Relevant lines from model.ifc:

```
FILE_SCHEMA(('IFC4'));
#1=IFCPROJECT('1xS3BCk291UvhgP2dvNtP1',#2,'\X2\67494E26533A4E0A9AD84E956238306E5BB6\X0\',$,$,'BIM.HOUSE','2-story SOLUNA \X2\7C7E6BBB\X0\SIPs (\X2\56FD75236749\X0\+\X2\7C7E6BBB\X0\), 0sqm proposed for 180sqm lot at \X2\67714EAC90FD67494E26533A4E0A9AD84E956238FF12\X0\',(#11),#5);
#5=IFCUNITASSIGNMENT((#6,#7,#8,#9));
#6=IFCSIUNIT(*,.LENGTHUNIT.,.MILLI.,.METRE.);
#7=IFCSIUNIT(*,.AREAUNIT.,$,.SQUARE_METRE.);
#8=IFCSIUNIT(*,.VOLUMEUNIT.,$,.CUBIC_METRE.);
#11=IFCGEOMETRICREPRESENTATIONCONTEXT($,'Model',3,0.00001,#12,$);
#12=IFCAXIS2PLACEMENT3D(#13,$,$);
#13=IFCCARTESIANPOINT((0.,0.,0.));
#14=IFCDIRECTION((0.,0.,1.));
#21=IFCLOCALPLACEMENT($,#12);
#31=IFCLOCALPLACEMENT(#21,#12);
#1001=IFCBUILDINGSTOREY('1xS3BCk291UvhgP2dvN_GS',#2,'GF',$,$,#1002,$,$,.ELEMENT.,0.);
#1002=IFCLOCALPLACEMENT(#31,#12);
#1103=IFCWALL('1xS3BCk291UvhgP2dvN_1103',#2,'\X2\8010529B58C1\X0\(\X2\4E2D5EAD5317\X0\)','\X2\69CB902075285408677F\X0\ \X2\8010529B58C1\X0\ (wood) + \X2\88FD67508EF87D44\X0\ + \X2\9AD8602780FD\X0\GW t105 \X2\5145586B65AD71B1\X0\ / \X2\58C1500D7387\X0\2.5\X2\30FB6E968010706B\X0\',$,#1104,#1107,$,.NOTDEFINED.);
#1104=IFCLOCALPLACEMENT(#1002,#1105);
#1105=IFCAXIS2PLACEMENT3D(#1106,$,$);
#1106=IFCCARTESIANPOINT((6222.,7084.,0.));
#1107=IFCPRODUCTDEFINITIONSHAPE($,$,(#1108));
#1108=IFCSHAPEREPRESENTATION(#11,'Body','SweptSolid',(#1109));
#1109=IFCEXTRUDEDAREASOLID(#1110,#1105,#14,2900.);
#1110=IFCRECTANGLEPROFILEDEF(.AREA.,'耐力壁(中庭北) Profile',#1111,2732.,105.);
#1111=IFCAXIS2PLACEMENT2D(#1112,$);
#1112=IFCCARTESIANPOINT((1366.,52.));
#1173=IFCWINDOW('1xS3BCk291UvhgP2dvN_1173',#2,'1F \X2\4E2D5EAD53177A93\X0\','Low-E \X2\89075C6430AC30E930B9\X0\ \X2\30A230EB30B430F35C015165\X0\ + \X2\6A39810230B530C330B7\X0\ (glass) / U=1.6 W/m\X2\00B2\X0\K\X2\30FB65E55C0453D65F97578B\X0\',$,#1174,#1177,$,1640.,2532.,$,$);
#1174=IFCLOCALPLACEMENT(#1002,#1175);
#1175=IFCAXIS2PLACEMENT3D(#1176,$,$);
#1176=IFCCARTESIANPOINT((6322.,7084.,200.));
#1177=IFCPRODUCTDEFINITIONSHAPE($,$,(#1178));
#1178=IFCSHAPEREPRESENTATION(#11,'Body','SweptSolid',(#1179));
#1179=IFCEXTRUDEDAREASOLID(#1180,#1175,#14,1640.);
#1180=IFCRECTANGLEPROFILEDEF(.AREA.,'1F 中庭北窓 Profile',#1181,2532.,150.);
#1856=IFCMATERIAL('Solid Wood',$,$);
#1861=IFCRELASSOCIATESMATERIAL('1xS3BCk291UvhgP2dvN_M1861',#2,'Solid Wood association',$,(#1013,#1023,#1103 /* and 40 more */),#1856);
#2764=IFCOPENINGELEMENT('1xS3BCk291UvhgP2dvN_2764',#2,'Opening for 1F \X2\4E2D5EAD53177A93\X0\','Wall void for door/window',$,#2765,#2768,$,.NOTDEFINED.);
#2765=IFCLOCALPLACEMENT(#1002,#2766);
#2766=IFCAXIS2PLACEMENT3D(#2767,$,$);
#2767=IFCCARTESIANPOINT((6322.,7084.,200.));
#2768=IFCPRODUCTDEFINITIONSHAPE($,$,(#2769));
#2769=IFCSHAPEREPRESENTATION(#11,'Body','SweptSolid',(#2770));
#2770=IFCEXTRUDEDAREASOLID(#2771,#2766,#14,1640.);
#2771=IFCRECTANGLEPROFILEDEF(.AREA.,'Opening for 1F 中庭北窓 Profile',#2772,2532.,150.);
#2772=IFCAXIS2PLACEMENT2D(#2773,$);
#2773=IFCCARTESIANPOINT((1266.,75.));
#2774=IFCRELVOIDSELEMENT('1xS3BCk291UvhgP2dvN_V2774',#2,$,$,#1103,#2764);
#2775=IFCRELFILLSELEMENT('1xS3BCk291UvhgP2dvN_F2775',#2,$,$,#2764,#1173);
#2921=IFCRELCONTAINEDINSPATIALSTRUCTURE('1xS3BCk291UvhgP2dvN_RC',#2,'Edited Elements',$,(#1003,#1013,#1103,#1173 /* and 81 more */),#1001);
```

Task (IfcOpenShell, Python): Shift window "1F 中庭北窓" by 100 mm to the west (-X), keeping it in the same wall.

```python
import ifcopenshell
import ifcopenshell.api.geometry
import ifcopenshell.util.placement

model = ifcopenshell.open("model.ifc")

window = model.by_guid("1xS3BCk291UvhgP2dvN_1173")
opening = window.FillsVoids[0].RelatingOpeningElement
wall = opening.VoidsElements[0].RelatingBuildingElement

wall_matrix = ifcopenshell.util.placement.get_local_placement(wall.ObjectPlacement)
shift = wall_matrix[:3, 0] * -100.0
before = ifcopenshell.util.placement.get_local_placement(window.ObjectPlacement)[:3, 3].copy()

# The window is not placed relative to its opening, so move both.
for product in (opening, window):
    matrix = ifcopenshell.util.placement.get_local_placement(product.ObjectPlacement)
    matrix[:3, 3] += shift
    ifcopenshell.api.geometry.edit_object_placement(model, product=product, matrix=matrix, is_si=False)

after = ifcopenshell.util.placement.get_local_placement(window.ObjectPlacement)[:3, 3]
print("window moved by", (after - before).round(3) + 0.0)

model.write("model_rev.ifc")
```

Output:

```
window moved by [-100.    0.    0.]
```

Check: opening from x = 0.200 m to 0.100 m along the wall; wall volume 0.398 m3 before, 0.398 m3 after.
